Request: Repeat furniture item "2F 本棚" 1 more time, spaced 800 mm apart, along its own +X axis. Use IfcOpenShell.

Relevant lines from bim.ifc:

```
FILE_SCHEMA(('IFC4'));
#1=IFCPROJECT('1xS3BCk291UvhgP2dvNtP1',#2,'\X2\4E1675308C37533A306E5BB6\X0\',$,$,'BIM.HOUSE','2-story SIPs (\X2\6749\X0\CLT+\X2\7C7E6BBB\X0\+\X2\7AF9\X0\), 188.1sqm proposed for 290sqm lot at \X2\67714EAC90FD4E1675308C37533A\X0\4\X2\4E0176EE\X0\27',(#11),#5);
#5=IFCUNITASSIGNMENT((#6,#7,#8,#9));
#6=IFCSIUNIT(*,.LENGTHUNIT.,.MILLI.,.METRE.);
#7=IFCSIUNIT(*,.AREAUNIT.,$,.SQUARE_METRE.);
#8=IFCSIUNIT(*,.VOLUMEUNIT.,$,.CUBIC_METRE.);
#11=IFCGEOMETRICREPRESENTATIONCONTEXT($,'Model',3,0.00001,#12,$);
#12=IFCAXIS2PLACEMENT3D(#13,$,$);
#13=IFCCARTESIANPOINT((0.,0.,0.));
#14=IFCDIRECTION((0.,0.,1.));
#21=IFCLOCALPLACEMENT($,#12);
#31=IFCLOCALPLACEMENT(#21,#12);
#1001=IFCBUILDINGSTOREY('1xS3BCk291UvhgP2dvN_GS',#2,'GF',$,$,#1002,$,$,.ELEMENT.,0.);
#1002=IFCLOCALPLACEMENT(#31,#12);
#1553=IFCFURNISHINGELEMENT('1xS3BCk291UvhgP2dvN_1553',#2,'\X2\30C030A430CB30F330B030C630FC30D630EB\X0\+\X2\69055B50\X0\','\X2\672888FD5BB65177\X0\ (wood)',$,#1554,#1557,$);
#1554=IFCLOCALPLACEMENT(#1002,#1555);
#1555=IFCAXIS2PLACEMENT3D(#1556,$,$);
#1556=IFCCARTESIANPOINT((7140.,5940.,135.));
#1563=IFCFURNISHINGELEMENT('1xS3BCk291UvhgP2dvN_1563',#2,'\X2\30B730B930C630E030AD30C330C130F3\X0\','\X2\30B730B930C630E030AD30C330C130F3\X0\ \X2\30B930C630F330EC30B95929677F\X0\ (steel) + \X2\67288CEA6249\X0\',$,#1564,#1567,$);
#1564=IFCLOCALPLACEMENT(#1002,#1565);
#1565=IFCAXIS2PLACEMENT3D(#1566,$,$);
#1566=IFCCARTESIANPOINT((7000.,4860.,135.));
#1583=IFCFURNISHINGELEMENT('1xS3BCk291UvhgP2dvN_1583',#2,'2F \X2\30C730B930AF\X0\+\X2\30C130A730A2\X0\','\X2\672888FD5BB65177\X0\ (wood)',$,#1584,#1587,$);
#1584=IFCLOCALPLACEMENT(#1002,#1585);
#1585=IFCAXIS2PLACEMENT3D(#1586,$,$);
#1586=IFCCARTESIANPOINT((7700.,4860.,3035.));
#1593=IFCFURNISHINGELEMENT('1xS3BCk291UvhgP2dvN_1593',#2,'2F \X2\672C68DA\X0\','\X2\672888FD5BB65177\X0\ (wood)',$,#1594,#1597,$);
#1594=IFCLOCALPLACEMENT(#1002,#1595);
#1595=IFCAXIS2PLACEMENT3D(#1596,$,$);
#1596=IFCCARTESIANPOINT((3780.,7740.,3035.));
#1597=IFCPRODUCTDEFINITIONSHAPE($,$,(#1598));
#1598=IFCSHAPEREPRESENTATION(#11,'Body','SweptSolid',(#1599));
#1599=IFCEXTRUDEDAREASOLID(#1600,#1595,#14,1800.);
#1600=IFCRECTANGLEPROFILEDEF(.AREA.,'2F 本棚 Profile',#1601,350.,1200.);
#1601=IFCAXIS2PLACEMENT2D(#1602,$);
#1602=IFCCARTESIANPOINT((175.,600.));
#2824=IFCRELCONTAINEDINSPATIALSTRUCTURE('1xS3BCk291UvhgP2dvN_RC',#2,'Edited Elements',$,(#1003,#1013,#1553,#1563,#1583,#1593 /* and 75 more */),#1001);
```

```python
import ifcopenshell
import ifcopenshell.api.geometry
import ifcopenshell.api.root
import ifcopenshell.util.element
import ifcopenshell.util.placement
import ifcopenshell.util.unit

model = ifcopenshell.open("bim.ifc")
unit_scale = ifcopenshell.util.unit.calculate_unit_scale(model)


def reuse_history(source, copy):
    """copy_class also copies each property set's owner history, people and application; keep the originals."""
    for rel in copy.IsDefinedBy:
        if rel.is_a("IfcRelDefinesByProperties") and (history := rel.RelatingPropertyDefinition.OwnerHistory):
            rel.RelatingPropertyDefinition.OwnerHistory = source.OwnerHistory
            ifcopenshell.util.element.remove_deep2(model, history)


source = model.by_guid("1xS3BCk291UvhgP2dvN_1593")
base = ifcopenshell.util.placement.get_local_placement(source.ObjectPlacement)
step = base[:3, 0] * 0.8 / unit_scale

for i in range(1, 2):
    copy = ifcopenshell.api.root.copy_class(model, product=source)
    copy.Representation = ifcopenshell.util.element.copy_deep(
        model, source.Representation, exclude=["IfcGeometricRepresentationContext", "IfcRepresentationMap"]
    )
    reuse_history(source, copy)
    matrix = base.copy()
    matrix[:3, 3] += i * step
    print("added at", matrix[:3, 3].round(3) + 0.0)
    ifcopenshell.api.geometry.edit_object_placement(model, product=copy, matrix=matrix, is_si=False)

model.write("bim_edited.ifc")
```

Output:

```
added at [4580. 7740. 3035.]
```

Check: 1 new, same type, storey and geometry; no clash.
